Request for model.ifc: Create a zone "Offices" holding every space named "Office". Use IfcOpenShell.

First a look at what the model holds.

```python
import ifcopenshell

model = ifcopenshell.open("model.ifc")
print(model.schema)
seen = {}
for space in model.by_type("IfcSpace"):
    seen[space.LongName] = seen.get(space.LongName, 0) + 1
for name, count in sorted(seen.items(), key=str):
    print(count, "x", name)
print("zones:", [z.Name for z in model.by_type("IfcZone")][:20])
```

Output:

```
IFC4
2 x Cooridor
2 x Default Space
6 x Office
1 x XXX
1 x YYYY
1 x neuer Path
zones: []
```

```python
import ifcopenshell
import ifcopenshell.api.group
import ifcopenshell.api.root

model = ifcopenshell.open("model.ifc")

names = {"Office"}
spaces = [s for s in model.by_type("IfcSpace") if s.LongName in names]

zone = ifcopenshell.api.root.create_entity(model, ifc_class="IfcZone", name="Offices")
ifcopenshell.api.group.assign_group(model, products=spaces, group=zone)
print(len(spaces), "spaces in", zone.Name)

model.write("model_v2.ifc")
```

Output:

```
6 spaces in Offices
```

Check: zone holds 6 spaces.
